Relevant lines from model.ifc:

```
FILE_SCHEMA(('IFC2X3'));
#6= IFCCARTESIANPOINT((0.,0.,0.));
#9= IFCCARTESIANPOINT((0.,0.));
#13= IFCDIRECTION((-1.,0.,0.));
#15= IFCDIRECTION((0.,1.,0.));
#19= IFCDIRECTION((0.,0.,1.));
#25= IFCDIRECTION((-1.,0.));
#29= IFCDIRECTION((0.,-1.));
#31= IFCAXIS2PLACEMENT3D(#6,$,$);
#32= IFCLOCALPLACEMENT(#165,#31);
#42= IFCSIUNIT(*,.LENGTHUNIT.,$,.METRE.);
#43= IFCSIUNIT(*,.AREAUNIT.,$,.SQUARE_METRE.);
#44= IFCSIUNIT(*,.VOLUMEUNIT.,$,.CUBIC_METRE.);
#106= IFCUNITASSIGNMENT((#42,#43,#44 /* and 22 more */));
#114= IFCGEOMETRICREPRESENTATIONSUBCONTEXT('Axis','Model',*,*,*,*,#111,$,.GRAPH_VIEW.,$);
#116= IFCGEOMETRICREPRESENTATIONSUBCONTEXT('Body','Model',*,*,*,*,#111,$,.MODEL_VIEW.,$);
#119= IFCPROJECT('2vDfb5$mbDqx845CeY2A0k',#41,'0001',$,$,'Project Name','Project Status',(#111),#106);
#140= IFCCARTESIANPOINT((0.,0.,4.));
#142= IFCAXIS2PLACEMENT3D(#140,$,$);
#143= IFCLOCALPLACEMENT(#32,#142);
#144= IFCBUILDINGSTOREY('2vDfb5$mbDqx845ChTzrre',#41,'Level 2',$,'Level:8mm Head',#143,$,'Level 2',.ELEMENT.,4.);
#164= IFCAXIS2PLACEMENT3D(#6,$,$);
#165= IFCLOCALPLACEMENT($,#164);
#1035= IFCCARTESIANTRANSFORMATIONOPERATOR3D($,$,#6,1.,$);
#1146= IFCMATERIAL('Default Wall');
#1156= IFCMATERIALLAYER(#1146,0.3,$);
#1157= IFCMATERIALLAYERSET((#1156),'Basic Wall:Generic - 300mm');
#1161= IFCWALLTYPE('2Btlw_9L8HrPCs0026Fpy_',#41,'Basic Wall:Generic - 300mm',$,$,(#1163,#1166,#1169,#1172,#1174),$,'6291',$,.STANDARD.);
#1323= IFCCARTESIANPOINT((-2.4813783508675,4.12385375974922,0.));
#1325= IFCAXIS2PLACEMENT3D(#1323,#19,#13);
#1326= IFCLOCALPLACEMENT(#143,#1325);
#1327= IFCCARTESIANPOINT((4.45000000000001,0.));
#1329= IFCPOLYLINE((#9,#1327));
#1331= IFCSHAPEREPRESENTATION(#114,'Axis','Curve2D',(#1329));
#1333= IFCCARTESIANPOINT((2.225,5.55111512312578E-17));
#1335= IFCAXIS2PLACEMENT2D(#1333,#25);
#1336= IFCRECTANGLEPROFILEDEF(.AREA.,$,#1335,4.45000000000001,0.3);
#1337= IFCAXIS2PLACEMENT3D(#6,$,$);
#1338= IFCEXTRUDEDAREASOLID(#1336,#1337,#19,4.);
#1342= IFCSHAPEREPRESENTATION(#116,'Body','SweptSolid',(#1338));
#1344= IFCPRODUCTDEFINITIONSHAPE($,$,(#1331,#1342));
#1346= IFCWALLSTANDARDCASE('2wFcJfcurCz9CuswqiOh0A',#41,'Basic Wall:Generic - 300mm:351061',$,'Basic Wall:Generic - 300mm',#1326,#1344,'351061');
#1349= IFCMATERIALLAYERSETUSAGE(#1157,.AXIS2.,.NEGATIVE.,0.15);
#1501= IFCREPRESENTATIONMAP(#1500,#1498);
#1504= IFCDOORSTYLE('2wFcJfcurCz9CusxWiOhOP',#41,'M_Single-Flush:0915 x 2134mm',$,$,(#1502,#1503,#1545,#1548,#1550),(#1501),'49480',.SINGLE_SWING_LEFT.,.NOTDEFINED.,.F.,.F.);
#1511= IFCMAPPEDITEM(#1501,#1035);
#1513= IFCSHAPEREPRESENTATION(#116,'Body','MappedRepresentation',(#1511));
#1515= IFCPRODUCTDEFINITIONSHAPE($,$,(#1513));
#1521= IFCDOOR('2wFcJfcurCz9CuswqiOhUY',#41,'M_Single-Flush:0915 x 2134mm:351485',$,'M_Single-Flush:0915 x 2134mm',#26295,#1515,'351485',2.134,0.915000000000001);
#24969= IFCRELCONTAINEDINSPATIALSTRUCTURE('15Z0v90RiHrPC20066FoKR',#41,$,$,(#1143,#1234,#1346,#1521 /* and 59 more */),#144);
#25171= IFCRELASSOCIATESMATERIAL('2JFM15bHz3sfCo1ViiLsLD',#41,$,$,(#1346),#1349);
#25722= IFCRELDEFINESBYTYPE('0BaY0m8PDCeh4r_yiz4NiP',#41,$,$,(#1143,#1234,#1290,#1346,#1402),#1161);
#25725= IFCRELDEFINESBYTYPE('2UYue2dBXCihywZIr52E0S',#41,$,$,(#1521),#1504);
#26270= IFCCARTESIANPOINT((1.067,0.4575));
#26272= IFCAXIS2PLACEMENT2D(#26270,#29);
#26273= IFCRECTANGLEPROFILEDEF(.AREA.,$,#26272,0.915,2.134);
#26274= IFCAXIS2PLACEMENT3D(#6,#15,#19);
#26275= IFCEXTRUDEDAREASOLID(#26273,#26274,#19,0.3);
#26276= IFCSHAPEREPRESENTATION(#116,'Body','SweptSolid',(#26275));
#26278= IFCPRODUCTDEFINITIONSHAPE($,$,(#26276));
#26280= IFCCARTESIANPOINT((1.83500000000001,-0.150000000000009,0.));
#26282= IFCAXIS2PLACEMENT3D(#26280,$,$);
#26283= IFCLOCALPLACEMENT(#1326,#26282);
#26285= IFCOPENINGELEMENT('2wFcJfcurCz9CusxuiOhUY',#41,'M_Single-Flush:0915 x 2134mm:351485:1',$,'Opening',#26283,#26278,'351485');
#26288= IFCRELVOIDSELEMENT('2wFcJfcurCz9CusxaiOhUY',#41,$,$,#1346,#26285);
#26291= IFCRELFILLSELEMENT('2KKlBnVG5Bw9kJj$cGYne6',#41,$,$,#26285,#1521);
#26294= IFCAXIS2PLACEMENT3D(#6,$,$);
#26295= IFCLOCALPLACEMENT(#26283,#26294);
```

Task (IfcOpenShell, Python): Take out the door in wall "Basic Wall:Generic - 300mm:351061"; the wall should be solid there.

```python
import ifcopenshell
import ifcopenshell.api.feature
import ifcopenshell.api.root
import ifcopenshell.geom
import ifcopenshell.util.shape

model = ifcopenshell.open("model.ifc")
settings = ifcopenshell.geom.settings()


def volume(element):
    """Net volume in cubic metres, openings subtracted."""
    shape = ifcopenshell.geom.create_shape(settings, element)
    return ifcopenshell.util.shape.get_volume(shape.geometry)


door = model.by_guid("2wFcJfcurCz9CuswqiOhUY")
opening = door.FillsVoids[0].RelatingOpeningElement
wall = opening.VoidsElements[0].RelatingBuildingElement
before = volume(wall)

ifcopenshell.api.root.remove_product(model, product=door)
ifcopenshell.api.feature.remove_feature(model, feature=opening)

after = volume(wall)

print(f"wall volume {before:.3f} -> {after:.3f} m3")

model.write("model_updated.ifc")
```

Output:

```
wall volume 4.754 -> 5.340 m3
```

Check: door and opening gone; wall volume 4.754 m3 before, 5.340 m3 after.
